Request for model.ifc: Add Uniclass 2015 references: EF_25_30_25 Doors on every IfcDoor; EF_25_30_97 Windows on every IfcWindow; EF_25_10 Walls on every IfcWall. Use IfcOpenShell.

First a look at what the model holds.

```python
import ifcopenshell

model = ifcopenshell.open("model.ifc")
print(model.schema)
print("classifications:", [c.Name for c in model.by_type("IfcClassification")])
for ifc_class in ("IfcDoor", "IfcRoof", "IfcStair", "IfcWall", "IfcWindow"):
    print(ifc_class, len(model.by_type(ifc_class)))
```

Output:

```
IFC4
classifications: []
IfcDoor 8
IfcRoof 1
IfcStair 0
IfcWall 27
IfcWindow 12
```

```python
import ifcopenshell
import ifcopenshell.api.classification

model = ifcopenshell.open("model.ifc")

system = ifcopenshell.api.classification.add_classification(model, classification="Uniclass 2015")

codes = {
    "IfcDoor": ("EF_25_30_25", "Doors"),
    "IfcWindow": ("EF_25_30_97", "Windows"),
    "IfcWall": ("EF_25_10", "Walls"),
}
for ifc_class, (code, name) in codes.items():
    products = model.by_type(ifc_class)
    ifcopenshell.api.classification.add_reference(
        model, products=products, classification=system, identification=code, name=name
    )
    print(code, len(products))

model.write("model-out.ifc")
```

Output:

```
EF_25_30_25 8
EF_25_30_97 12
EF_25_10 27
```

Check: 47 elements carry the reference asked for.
